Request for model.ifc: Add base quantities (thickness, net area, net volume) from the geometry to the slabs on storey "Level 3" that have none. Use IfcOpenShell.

First a look at what the model holds.

```python
import ifcopenshell
import ifcopenshell.util.element
import ifcopenshell.util.unit

model = ifcopenshell.open("model.ifc")
print(model.schema)
for unit_type in ("LENGTHUNIT", "AREAUNIT", "VOLUMEUNIT"):
    print(unit_type, ifcopenshell.util.unit.calculate_unit_scale(model, unit_type))
storey = next(s for s in model.by_type("IfcBuildingStorey") if s.Name == "Level 3")
slabs = [e for e in ifcopenshell.util.element.get_decomposition(storey) if e.is_a("IfcSlab")]
for e in sorted(slabs, key=lambda e: e.id()):
    print(e.id(), e.is_a(), e.Name, list(ifcopenshell.util.element.get_psets(e, qtos_only=True)), sep=" | ")
```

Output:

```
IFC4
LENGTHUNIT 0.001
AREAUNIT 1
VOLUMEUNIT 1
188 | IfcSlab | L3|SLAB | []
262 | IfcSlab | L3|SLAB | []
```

```python
import ifcopenshell
import ifcopenshell.api.pset
import ifcopenshell.geom
import ifcopenshell.util.element
import ifcopenshell.util.shape
import ifcopenshell.util.unit

model = ifcopenshell.open("model.ifc")
unit_scale = ifcopenshell.util.unit.calculate_unit_scale(model)
area_scale = ifcopenshell.util.unit.calculate_unit_scale(model, "AREAUNIT")
volume_scale = ifcopenshell.util.unit.calculate_unit_scale(model, "VOLUMEUNIT")
settings = ifcopenshell.geom.settings()

storey = next(s for s in model.by_type("IfcBuildingStorey") if s.Name == "Level 3")
slabs = [e for e in ifcopenshell.util.element.get_decomposition(storey) if e.is_a("IfcSlab")]

for e in sorted(slabs, key=lambda e: e.id()):
    if ifcopenshell.util.element.get_psets(e, qtos_only=True, should_inherit=False):
        continue
    # Geometry comes back in metres, in the element's own axes.
    shape = ifcopenshell.geom.create_shape(settings, e)
    values = {
        "Width": ifcopenshell.util.shape.get_z(shape.geometry) / unit_scale,
        "NetArea": ifcopenshell.util.shape.get_footprint_area(shape.geometry) / area_scale,
        "NetVolume": ifcopenshell.util.shape.get_volume(shape.geometry) / volume_scale,
    }
    qto = ifcopenshell.api.pset.add_qto(model, product=e, name="Qto_SlabBaseQuantities")
    ifcopenshell.api.pset.edit_qto(model, qto=qto, properties=values)
    print(e.id(), {k: round(v, 3) for k, v in values.items()})

model.write("model_v2.ifc")
```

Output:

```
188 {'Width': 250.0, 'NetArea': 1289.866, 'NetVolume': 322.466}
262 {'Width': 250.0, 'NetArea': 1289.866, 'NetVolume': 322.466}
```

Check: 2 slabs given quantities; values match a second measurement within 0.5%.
